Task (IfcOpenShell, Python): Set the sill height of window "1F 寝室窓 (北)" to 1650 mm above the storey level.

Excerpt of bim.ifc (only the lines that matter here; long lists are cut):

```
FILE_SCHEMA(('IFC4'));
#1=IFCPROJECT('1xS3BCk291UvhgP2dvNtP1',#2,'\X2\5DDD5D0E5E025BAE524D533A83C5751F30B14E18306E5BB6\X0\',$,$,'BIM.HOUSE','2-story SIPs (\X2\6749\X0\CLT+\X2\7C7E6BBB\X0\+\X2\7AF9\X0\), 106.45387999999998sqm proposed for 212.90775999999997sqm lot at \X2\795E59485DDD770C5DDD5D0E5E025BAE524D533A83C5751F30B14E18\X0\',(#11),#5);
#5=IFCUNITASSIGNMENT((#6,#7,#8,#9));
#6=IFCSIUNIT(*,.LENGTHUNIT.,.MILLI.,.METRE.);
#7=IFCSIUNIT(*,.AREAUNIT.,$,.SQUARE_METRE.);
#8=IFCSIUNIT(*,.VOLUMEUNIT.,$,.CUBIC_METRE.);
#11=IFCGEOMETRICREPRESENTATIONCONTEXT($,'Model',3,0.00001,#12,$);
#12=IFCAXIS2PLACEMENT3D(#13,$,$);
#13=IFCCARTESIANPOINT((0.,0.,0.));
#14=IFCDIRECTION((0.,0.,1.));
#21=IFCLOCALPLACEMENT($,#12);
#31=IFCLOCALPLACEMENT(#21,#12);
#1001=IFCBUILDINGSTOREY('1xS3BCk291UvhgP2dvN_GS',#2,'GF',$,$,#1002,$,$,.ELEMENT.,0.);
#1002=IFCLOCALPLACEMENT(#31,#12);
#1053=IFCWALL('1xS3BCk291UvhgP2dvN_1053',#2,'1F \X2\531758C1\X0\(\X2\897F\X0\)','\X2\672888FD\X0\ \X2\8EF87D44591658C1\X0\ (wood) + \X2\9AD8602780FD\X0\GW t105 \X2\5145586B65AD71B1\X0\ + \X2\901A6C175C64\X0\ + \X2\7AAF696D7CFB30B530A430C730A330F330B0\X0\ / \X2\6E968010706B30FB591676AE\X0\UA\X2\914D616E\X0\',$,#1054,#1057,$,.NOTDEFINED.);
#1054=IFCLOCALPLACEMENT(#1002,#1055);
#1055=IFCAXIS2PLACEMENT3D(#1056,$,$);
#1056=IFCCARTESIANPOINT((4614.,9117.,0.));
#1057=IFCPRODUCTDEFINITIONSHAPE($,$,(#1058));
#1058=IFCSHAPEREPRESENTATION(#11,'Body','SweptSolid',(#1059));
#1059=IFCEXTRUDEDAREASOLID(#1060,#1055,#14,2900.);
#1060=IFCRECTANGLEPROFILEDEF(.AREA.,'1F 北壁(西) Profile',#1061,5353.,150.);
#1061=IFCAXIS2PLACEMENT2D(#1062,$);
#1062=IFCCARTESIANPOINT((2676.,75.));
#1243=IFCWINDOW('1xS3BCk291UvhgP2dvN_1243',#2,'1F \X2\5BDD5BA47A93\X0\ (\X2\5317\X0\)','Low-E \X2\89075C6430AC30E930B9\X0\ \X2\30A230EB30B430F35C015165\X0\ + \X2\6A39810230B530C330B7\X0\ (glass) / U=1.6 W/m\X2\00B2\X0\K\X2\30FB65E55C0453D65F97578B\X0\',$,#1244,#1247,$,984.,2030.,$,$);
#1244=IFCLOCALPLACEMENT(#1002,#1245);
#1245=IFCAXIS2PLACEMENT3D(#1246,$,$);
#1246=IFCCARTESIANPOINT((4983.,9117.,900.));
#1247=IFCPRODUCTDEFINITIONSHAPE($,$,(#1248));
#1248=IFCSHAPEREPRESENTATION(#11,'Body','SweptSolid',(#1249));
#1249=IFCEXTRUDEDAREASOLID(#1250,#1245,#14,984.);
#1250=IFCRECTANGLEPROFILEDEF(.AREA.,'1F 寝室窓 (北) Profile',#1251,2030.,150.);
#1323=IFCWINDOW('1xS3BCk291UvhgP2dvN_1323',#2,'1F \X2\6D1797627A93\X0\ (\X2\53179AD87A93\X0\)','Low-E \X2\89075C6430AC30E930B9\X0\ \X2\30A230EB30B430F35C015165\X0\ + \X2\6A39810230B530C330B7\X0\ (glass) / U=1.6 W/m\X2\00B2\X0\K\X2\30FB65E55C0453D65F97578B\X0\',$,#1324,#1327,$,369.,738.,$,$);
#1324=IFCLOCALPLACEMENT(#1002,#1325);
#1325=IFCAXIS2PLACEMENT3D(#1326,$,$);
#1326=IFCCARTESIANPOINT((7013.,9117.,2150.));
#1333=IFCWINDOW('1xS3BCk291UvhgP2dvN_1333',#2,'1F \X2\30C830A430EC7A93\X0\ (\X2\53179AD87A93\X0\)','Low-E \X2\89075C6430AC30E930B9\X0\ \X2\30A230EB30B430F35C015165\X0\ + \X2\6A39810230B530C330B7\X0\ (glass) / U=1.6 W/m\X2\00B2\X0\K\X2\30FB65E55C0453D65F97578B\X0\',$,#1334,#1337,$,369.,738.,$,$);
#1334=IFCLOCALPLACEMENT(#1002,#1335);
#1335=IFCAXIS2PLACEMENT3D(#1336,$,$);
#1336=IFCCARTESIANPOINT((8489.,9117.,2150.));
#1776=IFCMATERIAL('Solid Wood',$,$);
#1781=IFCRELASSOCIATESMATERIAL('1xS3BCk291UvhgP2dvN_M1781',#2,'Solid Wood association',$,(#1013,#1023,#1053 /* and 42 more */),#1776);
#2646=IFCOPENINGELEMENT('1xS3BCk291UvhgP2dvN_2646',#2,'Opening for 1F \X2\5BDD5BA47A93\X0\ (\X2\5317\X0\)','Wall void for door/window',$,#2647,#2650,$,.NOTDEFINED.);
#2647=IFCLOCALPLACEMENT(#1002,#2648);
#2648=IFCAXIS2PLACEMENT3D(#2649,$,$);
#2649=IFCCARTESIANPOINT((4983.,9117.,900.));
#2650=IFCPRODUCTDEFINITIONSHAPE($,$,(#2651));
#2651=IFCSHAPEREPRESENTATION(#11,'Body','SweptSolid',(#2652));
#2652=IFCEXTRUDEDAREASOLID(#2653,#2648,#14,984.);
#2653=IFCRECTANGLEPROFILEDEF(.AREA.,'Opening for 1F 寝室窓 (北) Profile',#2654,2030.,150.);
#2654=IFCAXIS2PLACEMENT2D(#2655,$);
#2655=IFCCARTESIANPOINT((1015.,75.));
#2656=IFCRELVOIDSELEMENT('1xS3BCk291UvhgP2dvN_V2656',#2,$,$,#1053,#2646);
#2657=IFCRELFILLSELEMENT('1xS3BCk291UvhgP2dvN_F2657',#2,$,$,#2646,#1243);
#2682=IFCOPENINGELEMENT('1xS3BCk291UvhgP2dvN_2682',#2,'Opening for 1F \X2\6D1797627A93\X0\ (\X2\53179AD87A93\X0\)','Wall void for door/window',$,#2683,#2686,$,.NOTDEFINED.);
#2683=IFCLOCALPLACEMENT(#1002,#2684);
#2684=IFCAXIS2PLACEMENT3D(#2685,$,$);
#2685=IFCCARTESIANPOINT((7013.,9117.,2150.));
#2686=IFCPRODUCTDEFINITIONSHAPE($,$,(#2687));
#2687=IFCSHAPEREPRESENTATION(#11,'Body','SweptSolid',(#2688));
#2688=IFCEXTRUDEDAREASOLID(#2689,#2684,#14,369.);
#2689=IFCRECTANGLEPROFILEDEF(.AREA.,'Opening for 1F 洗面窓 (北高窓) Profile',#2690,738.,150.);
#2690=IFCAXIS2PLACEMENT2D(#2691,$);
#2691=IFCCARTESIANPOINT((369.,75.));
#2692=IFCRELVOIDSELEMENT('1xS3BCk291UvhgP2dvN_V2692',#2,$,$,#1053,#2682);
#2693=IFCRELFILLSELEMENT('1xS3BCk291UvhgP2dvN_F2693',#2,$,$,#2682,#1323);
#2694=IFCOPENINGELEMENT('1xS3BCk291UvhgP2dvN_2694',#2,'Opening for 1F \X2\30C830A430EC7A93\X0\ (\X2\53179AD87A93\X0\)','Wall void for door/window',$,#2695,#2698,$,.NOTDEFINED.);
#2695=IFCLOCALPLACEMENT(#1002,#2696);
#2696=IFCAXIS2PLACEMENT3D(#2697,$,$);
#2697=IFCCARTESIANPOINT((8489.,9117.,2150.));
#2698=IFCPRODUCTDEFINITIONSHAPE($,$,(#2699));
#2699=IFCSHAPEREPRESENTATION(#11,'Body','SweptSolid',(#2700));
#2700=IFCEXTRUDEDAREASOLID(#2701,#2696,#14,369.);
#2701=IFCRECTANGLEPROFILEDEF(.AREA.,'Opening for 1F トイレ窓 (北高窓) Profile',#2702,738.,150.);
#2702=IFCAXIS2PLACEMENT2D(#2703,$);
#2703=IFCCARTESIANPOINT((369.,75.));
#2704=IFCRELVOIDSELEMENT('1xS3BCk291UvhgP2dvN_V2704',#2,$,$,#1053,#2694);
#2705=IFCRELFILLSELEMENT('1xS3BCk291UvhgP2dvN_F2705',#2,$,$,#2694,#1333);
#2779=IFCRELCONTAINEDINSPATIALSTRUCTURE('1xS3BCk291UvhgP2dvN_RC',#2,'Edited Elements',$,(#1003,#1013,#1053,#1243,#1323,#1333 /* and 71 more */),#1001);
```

```python
import numpy as np
import ifcopenshell
import ifcopenshell.api.geometry
import ifcopenshell.geom
import ifcopenshell.util.element
import ifcopenshell.util.placement
import ifcopenshell.util.shape
import ifcopenshell.util.unit

model = ifcopenshell.open("bim.ifc")
unit_scale = ifcopenshell.util.unit.calculate_unit_scale(model)

window = model.by_id(1243)
opening = window.FillsVoids[0].RelatingOpeningElement
storey = ifcopenshell.util.element.get_container(window, ifc_class="IfcBuildingStorey")
level = ifcopenshell.util.placement.get_local_placement(storey.ObjectPlacement)[2, 3]

# The opening's origin need not be at the sill, so measure its lowest point.
shape = ifcopenshell.geom.create_shape(ifcopenshell.geom.settings(), opening)
bottom = ifcopenshell.util.shape.get_shape_bottom_elevation(shape, shape.geometry) / unit_scale
dz = level + 1650.0 - bottom

shift = np.array([0.0, 0.0, dz])
# The window is not placed relative to its opening, so move both.
for product in (opening, window):
    matrix = ifcopenshell.util.placement.get_local_placement(product.ObjectPlacement)
    matrix[:3, 3] += shift
    ifcopenshell.api.geometry.edit_object_placement(model, product=product, matrix=matrix, is_si=False)

print(f"moved by {dz * unit_scale:+.3f} m")

model.write("bim_v2.ifc")
```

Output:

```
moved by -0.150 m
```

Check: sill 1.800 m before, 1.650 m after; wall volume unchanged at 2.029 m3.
